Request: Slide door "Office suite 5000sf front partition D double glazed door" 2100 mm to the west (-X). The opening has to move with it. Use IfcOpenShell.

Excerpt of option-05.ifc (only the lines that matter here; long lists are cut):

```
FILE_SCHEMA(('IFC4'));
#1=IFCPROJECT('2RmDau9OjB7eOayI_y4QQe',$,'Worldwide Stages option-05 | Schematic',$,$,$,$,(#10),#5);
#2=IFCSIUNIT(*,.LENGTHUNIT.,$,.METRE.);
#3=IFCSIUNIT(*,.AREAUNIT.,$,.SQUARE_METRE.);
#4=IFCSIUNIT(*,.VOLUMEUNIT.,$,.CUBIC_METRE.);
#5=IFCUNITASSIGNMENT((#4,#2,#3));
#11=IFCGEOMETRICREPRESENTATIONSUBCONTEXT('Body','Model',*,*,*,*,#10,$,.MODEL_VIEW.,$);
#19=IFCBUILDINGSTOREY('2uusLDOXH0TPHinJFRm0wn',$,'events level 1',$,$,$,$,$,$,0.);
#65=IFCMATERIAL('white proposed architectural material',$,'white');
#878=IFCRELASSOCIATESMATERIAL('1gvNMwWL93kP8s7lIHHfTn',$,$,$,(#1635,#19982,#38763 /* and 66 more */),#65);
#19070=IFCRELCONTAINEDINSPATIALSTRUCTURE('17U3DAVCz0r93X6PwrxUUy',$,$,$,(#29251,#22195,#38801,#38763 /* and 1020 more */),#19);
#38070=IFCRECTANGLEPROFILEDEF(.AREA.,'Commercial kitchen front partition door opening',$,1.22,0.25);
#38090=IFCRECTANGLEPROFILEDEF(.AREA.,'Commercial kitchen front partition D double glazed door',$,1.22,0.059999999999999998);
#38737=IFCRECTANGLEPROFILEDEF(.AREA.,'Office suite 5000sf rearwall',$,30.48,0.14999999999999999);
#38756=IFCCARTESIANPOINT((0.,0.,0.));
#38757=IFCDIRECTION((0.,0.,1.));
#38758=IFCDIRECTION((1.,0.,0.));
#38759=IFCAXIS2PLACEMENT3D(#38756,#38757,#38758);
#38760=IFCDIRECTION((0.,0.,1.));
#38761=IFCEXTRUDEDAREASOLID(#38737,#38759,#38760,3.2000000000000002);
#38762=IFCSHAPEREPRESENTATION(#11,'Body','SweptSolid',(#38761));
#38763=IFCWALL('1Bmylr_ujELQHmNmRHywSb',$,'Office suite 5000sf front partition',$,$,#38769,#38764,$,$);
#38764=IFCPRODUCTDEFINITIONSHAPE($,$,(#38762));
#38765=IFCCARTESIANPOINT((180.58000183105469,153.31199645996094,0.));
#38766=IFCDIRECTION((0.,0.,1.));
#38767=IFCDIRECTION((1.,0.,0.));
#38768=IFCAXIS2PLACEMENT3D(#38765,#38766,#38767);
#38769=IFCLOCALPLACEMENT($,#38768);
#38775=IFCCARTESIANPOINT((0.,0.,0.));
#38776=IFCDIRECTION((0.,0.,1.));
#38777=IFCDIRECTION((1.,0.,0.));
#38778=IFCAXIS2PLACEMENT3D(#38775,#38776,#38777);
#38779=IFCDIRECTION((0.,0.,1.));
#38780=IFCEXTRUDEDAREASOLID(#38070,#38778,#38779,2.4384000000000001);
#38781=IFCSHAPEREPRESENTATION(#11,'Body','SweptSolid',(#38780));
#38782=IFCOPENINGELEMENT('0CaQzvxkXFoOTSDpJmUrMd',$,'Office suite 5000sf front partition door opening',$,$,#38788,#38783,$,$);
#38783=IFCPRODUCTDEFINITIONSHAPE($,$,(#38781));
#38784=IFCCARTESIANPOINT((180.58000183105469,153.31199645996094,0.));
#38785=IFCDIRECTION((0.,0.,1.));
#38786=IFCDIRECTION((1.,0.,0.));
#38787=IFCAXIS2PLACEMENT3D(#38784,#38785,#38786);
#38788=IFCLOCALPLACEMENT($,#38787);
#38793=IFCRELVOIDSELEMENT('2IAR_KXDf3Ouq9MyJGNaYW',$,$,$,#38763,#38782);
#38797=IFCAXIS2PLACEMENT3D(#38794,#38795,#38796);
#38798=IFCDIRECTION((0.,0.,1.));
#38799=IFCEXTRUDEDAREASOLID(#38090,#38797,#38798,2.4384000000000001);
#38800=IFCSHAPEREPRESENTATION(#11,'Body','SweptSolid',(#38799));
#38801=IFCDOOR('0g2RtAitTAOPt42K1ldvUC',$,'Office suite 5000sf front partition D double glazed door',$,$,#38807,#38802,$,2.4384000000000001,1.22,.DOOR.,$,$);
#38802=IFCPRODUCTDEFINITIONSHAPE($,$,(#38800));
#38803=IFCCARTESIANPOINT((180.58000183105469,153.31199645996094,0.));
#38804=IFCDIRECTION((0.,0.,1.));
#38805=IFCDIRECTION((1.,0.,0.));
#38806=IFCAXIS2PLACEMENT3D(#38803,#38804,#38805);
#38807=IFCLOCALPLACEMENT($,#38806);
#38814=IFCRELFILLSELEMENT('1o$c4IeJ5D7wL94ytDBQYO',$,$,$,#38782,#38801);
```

```python
import ifcopenshell
import ifcopenshell.api.geometry
import ifcopenshell.util.placement

model = ifcopenshell.open("option-05.ifc")

door = model.by_guid("0g2RtAitTAOPt42K1ldvUC")
opening = door.FillsVoids[0].RelatingOpeningElement
wall = opening.VoidsElements[0].RelatingBuildingElement

wall_matrix = ifcopenshell.util.placement.get_local_placement(wall.ObjectPlacement)
shift = wall_matrix[:3, 0] * -2.1
before = ifcopenshell.util.placement.get_local_placement(door.ObjectPlacement)[:3, 3].copy()

# The door is not placed relative to its opening, so move both.
for product in (opening, door):
    matrix = ifcopenshell.util.placement.get_local_placement(product.ObjectPlacement)
    matrix[:3, 3] += shift
    ifcopenshell.api.geometry.edit_object_placement(model, product=product, matrix=matrix, is_si=False)

after = ifcopenshell.util.placement.get_local_placement(door.ObjectPlacement)[:3, 3]
print("door moved by", (after - before).round(3) + 0.0)

model.write("option-05_v2.ifc")
```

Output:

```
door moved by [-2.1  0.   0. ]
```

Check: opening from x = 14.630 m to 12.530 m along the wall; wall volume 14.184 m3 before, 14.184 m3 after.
